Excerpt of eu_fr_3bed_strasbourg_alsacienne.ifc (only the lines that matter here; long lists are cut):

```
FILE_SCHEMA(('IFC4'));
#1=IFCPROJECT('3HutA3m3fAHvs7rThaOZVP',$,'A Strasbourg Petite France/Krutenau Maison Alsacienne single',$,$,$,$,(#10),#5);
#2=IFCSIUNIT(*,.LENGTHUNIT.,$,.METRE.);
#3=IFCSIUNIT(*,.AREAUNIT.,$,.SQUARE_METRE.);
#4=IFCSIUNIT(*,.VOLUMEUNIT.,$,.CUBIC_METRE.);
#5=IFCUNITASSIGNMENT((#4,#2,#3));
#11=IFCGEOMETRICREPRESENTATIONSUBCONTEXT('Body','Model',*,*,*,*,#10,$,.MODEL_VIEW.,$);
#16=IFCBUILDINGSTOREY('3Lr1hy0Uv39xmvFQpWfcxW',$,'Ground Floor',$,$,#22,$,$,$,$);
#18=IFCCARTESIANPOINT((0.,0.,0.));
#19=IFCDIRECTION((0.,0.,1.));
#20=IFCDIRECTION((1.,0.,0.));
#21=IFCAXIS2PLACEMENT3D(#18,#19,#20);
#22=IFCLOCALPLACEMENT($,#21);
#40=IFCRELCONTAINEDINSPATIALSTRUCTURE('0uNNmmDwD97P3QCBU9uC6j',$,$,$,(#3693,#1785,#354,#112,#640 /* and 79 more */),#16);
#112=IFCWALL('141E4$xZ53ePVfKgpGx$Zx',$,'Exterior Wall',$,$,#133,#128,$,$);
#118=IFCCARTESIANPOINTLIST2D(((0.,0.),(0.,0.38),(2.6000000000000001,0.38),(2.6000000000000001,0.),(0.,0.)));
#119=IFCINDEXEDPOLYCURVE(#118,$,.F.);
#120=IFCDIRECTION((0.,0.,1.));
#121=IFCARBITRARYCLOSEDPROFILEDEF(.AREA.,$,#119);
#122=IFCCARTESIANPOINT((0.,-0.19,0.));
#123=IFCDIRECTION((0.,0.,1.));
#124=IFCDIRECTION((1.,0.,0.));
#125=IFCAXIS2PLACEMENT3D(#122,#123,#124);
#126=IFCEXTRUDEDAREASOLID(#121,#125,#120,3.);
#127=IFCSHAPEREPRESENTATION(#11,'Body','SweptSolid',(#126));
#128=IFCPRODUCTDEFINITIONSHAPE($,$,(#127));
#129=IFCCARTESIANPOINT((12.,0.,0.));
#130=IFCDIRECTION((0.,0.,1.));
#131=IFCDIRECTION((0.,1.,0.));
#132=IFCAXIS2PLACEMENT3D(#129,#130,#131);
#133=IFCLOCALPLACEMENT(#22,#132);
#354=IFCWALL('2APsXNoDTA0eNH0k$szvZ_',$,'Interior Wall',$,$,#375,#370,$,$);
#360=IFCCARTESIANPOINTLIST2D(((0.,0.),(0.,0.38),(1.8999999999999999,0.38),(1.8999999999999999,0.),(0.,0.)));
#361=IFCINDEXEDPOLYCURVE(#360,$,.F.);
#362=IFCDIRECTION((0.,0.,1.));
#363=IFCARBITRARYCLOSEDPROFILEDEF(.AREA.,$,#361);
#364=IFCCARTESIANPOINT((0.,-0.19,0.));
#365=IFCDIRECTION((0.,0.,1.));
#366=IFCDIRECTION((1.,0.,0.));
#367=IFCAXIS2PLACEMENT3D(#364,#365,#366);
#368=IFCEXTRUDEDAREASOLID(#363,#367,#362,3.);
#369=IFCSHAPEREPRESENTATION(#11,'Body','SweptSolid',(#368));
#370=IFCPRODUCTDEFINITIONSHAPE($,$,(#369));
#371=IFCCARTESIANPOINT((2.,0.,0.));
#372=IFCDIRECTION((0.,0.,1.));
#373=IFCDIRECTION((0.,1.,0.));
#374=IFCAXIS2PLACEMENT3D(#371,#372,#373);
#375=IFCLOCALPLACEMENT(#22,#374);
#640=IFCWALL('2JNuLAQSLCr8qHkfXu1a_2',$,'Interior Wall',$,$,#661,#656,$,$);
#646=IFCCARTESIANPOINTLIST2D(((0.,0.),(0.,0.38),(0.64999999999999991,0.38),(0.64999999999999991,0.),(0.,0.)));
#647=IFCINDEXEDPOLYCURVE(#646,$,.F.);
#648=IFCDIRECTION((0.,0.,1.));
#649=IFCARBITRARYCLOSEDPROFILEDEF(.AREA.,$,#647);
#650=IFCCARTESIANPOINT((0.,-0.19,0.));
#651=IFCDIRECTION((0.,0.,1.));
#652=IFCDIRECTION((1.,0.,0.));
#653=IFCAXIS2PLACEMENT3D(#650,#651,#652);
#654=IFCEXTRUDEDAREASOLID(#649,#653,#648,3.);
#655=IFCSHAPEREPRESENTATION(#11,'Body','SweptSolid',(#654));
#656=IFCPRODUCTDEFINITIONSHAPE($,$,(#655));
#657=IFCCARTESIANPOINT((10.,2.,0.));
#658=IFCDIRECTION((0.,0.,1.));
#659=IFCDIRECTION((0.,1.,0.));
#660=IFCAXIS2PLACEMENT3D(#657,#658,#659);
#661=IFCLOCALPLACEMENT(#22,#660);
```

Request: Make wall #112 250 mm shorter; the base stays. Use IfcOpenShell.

```python
import ifcopenshell
import ifcopenshell.geom
import ifcopenshell.util.representation
import ifcopenshell.util.shape
import ifcopenshell.util.unit

model = ifcopenshell.open("eu_fr_3bed_strasbourg_alsacienne.ifc")
unit_scale = ifcopenshell.util.unit.calculate_unit_scale(model)
settings = ifcopenshell.geom.settings()


def volume(element):
    """Net volume in cubic metres, openings subtracted."""
    shape = ifcopenshell.geom.create_shape(settings, element)
    return ifcopenshell.util.shape.get_volume(shape.geometry)


wall = model.by_guid("141E4$xZ53ePVfKgpGx$Zx")
before = volume(wall)

body = ifcopenshell.util.representation.get_representation(wall, "Model", "Body")
solid = body.Items[0]
old_height = solid.Depth
solid.Depth -= 0.25 / unit_scale
after = volume(wall)

print(f"height {old_height:g} -> {solid.Depth:g}, volume {before:.3f} -> {after:.3f} m3")

model.write("eu_fr_3bed_strasbourg_alsacienne_v2.ifc")
```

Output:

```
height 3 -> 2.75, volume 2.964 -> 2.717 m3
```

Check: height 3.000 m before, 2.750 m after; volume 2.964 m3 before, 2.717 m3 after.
